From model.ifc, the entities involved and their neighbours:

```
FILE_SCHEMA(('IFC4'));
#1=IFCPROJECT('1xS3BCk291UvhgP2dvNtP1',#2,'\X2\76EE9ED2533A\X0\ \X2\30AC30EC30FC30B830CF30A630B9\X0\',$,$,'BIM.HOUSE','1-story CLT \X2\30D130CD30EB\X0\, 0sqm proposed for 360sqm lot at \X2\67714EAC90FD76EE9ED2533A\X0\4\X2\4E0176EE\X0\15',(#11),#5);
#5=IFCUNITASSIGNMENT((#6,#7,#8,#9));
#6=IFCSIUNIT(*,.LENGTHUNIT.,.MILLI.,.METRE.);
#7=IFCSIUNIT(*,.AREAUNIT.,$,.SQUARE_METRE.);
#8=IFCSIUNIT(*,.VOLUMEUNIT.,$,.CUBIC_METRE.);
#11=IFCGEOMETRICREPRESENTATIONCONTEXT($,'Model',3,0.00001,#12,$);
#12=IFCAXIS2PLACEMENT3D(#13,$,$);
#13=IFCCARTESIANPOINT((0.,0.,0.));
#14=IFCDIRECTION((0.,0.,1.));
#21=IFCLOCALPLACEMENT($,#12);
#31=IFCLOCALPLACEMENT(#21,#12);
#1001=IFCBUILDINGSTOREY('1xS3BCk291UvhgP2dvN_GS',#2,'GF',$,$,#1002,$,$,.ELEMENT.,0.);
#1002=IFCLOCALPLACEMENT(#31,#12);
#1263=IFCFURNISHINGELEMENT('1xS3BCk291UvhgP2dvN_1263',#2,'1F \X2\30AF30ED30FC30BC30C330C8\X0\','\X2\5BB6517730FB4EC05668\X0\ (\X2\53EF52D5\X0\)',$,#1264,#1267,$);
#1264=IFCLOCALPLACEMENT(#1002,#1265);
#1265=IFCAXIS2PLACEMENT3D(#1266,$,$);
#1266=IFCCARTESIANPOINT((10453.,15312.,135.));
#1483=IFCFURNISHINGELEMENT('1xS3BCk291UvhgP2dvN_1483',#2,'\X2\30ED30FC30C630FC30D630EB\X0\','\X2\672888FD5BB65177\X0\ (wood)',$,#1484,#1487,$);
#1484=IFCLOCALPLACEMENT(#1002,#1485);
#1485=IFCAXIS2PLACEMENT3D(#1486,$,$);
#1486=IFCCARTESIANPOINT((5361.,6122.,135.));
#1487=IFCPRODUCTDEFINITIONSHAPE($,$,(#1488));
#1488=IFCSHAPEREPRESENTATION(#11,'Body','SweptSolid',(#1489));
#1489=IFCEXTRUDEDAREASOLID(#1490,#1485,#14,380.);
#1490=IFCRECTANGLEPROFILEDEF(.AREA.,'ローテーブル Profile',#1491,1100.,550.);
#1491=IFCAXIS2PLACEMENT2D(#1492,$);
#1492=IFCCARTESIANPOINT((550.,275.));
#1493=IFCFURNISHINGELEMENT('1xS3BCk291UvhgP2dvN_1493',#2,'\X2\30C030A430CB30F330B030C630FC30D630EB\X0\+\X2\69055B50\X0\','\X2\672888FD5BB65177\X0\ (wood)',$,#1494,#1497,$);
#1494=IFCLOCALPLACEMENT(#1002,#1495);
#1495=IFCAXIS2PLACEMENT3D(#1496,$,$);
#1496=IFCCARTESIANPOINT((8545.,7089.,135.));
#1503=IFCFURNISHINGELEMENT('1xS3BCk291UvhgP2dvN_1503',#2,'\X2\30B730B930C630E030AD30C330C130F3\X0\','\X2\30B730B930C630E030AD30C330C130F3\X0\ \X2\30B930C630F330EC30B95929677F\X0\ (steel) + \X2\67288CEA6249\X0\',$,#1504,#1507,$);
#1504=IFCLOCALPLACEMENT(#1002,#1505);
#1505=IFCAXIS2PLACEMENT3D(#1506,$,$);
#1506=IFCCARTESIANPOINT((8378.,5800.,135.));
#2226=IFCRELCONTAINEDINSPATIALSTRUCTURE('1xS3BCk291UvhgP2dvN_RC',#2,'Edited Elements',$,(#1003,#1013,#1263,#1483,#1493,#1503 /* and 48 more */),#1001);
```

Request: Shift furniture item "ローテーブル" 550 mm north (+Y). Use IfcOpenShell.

```python
import ifcopenshell
import ifcopenshell.api.geometry
import ifcopenshell.util.placement

model = ifcopenshell.open("model.ifc")

item = model.by_guid("1xS3BCk291UvhgP2dvN_1483")
matrix = ifcopenshell.util.placement.get_local_placement(item.ObjectPlacement)
matrix[1, 3] += 550.0
ifcopenshell.api.geometry.edit_object_placement(model, product=item, matrix=matrix, is_si=False)

print(ifcopenshell.util.placement.get_local_placement(item.ObjectPlacement).round(3) + 0.0)

model.write("model-out.ifc")
```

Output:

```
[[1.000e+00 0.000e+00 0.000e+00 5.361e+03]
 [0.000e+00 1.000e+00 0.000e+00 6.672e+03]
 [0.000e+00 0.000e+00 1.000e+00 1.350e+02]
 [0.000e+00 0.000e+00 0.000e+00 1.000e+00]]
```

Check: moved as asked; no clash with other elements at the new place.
